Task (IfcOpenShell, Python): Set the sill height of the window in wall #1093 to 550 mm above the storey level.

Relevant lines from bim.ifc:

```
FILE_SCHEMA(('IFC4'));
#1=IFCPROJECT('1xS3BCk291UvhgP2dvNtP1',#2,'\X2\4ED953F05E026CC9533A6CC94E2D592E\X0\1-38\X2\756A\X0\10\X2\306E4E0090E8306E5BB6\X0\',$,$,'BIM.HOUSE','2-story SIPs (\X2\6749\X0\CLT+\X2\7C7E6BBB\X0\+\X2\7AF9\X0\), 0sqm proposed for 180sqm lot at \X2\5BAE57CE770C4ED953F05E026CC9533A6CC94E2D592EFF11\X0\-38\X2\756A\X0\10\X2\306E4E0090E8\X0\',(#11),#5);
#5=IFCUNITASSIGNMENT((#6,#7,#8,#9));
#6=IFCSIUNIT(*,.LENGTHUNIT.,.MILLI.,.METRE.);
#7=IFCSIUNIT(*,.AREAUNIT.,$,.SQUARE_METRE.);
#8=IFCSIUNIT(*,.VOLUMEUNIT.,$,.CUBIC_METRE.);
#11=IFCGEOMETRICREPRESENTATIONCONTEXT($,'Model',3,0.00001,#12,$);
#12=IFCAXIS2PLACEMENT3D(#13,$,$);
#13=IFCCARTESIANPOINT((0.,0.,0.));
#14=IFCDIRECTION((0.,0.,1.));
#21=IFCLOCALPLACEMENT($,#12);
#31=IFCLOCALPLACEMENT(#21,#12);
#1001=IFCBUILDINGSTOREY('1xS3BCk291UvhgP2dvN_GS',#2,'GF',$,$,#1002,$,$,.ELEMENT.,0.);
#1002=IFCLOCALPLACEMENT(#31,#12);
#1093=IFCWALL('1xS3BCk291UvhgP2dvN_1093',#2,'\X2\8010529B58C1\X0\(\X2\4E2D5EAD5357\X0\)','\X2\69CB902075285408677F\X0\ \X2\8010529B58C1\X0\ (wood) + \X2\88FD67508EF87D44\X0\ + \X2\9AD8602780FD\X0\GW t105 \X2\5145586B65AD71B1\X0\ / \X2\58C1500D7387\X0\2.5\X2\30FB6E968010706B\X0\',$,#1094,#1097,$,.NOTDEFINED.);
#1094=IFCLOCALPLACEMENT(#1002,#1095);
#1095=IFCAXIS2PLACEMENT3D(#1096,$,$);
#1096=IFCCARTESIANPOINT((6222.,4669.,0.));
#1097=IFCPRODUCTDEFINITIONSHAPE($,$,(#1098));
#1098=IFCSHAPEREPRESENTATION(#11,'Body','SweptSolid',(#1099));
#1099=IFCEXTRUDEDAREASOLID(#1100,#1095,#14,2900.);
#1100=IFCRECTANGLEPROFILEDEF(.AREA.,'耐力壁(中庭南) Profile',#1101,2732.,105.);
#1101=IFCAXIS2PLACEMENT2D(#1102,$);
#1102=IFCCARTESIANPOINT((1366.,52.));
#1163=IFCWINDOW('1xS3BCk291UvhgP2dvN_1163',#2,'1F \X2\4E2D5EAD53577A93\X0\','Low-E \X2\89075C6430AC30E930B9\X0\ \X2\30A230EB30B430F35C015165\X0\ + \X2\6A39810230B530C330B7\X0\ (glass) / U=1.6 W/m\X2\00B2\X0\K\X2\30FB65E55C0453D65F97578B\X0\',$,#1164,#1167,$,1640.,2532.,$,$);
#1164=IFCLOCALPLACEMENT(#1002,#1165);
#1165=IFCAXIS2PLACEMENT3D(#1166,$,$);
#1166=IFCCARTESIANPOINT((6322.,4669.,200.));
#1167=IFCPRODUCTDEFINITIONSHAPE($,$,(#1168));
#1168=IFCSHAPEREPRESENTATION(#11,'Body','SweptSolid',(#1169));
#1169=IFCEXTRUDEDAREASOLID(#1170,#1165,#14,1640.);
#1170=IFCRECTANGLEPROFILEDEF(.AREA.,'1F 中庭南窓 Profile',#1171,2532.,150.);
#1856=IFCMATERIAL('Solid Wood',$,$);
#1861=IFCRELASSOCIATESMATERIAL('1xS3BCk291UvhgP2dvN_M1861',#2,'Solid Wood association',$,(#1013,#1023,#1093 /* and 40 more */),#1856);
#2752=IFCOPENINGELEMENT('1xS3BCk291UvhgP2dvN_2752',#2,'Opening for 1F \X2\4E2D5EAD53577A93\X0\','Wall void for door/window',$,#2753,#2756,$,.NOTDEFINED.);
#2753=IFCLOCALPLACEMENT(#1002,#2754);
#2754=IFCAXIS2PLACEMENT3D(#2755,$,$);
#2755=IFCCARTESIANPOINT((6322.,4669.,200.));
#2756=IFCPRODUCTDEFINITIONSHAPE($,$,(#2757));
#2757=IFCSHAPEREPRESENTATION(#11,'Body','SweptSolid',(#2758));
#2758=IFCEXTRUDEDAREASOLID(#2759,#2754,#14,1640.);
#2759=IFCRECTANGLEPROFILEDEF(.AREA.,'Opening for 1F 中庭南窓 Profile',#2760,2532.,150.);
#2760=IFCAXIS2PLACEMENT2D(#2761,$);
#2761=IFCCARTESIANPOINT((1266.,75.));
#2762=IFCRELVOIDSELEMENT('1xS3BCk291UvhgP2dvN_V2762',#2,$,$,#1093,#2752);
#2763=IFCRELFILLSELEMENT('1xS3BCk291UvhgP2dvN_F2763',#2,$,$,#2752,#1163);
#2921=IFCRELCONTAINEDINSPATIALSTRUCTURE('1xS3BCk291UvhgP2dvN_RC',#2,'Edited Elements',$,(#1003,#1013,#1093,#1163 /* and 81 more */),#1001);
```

```python
import numpy as np
import ifcopenshell
import ifcopenshell.api.geometry
import ifcopenshell.geom
import ifcopenshell.util.element
import ifcopenshell.util.placement
import ifcopenshell.util.shape
import ifcopenshell.util.unit

model = ifcopenshell.open("bim.ifc")
unit_scale = ifcopenshell.util.unit.calculate_unit_scale(model)

window = model.by_guid("1xS3BCk291UvhgP2dvN_1163")
opening = window.FillsVoids[0].RelatingOpeningElement
storey = ifcopenshell.util.element.get_container(window, ifc_class="IfcBuildingStorey")
level = ifcopenshell.util.placement.get_local_placement(storey.ObjectPlacement)[2, 3]

# The opening's origin need not be at the sill, so measure its lowest point.
shape = ifcopenshell.geom.create_shape(ifcopenshell.geom.settings(), opening)
bottom = ifcopenshell.util.shape.get_shape_bottom_elevation(shape, shape.geometry) / unit_scale
dz = level + 0.55 / unit_scale - bottom

shift = np.array([0.0, 0.0, dz])
# The window is not placed relative to its opening, so move both.
for product in (opening, window):
    matrix = ifcopenshell.util.placement.get_local_placement(product.ObjectPlacement)
    matrix[:3, 3] += shift
    ifcopenshell.api.geometry.edit_object_placement(model, product=product, matrix=matrix, is_si=False)

print(f"moved by {dz * unit_scale:+.3f} m")

model.write("bim_updated.ifc")
```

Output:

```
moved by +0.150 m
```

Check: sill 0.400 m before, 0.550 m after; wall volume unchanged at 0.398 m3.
